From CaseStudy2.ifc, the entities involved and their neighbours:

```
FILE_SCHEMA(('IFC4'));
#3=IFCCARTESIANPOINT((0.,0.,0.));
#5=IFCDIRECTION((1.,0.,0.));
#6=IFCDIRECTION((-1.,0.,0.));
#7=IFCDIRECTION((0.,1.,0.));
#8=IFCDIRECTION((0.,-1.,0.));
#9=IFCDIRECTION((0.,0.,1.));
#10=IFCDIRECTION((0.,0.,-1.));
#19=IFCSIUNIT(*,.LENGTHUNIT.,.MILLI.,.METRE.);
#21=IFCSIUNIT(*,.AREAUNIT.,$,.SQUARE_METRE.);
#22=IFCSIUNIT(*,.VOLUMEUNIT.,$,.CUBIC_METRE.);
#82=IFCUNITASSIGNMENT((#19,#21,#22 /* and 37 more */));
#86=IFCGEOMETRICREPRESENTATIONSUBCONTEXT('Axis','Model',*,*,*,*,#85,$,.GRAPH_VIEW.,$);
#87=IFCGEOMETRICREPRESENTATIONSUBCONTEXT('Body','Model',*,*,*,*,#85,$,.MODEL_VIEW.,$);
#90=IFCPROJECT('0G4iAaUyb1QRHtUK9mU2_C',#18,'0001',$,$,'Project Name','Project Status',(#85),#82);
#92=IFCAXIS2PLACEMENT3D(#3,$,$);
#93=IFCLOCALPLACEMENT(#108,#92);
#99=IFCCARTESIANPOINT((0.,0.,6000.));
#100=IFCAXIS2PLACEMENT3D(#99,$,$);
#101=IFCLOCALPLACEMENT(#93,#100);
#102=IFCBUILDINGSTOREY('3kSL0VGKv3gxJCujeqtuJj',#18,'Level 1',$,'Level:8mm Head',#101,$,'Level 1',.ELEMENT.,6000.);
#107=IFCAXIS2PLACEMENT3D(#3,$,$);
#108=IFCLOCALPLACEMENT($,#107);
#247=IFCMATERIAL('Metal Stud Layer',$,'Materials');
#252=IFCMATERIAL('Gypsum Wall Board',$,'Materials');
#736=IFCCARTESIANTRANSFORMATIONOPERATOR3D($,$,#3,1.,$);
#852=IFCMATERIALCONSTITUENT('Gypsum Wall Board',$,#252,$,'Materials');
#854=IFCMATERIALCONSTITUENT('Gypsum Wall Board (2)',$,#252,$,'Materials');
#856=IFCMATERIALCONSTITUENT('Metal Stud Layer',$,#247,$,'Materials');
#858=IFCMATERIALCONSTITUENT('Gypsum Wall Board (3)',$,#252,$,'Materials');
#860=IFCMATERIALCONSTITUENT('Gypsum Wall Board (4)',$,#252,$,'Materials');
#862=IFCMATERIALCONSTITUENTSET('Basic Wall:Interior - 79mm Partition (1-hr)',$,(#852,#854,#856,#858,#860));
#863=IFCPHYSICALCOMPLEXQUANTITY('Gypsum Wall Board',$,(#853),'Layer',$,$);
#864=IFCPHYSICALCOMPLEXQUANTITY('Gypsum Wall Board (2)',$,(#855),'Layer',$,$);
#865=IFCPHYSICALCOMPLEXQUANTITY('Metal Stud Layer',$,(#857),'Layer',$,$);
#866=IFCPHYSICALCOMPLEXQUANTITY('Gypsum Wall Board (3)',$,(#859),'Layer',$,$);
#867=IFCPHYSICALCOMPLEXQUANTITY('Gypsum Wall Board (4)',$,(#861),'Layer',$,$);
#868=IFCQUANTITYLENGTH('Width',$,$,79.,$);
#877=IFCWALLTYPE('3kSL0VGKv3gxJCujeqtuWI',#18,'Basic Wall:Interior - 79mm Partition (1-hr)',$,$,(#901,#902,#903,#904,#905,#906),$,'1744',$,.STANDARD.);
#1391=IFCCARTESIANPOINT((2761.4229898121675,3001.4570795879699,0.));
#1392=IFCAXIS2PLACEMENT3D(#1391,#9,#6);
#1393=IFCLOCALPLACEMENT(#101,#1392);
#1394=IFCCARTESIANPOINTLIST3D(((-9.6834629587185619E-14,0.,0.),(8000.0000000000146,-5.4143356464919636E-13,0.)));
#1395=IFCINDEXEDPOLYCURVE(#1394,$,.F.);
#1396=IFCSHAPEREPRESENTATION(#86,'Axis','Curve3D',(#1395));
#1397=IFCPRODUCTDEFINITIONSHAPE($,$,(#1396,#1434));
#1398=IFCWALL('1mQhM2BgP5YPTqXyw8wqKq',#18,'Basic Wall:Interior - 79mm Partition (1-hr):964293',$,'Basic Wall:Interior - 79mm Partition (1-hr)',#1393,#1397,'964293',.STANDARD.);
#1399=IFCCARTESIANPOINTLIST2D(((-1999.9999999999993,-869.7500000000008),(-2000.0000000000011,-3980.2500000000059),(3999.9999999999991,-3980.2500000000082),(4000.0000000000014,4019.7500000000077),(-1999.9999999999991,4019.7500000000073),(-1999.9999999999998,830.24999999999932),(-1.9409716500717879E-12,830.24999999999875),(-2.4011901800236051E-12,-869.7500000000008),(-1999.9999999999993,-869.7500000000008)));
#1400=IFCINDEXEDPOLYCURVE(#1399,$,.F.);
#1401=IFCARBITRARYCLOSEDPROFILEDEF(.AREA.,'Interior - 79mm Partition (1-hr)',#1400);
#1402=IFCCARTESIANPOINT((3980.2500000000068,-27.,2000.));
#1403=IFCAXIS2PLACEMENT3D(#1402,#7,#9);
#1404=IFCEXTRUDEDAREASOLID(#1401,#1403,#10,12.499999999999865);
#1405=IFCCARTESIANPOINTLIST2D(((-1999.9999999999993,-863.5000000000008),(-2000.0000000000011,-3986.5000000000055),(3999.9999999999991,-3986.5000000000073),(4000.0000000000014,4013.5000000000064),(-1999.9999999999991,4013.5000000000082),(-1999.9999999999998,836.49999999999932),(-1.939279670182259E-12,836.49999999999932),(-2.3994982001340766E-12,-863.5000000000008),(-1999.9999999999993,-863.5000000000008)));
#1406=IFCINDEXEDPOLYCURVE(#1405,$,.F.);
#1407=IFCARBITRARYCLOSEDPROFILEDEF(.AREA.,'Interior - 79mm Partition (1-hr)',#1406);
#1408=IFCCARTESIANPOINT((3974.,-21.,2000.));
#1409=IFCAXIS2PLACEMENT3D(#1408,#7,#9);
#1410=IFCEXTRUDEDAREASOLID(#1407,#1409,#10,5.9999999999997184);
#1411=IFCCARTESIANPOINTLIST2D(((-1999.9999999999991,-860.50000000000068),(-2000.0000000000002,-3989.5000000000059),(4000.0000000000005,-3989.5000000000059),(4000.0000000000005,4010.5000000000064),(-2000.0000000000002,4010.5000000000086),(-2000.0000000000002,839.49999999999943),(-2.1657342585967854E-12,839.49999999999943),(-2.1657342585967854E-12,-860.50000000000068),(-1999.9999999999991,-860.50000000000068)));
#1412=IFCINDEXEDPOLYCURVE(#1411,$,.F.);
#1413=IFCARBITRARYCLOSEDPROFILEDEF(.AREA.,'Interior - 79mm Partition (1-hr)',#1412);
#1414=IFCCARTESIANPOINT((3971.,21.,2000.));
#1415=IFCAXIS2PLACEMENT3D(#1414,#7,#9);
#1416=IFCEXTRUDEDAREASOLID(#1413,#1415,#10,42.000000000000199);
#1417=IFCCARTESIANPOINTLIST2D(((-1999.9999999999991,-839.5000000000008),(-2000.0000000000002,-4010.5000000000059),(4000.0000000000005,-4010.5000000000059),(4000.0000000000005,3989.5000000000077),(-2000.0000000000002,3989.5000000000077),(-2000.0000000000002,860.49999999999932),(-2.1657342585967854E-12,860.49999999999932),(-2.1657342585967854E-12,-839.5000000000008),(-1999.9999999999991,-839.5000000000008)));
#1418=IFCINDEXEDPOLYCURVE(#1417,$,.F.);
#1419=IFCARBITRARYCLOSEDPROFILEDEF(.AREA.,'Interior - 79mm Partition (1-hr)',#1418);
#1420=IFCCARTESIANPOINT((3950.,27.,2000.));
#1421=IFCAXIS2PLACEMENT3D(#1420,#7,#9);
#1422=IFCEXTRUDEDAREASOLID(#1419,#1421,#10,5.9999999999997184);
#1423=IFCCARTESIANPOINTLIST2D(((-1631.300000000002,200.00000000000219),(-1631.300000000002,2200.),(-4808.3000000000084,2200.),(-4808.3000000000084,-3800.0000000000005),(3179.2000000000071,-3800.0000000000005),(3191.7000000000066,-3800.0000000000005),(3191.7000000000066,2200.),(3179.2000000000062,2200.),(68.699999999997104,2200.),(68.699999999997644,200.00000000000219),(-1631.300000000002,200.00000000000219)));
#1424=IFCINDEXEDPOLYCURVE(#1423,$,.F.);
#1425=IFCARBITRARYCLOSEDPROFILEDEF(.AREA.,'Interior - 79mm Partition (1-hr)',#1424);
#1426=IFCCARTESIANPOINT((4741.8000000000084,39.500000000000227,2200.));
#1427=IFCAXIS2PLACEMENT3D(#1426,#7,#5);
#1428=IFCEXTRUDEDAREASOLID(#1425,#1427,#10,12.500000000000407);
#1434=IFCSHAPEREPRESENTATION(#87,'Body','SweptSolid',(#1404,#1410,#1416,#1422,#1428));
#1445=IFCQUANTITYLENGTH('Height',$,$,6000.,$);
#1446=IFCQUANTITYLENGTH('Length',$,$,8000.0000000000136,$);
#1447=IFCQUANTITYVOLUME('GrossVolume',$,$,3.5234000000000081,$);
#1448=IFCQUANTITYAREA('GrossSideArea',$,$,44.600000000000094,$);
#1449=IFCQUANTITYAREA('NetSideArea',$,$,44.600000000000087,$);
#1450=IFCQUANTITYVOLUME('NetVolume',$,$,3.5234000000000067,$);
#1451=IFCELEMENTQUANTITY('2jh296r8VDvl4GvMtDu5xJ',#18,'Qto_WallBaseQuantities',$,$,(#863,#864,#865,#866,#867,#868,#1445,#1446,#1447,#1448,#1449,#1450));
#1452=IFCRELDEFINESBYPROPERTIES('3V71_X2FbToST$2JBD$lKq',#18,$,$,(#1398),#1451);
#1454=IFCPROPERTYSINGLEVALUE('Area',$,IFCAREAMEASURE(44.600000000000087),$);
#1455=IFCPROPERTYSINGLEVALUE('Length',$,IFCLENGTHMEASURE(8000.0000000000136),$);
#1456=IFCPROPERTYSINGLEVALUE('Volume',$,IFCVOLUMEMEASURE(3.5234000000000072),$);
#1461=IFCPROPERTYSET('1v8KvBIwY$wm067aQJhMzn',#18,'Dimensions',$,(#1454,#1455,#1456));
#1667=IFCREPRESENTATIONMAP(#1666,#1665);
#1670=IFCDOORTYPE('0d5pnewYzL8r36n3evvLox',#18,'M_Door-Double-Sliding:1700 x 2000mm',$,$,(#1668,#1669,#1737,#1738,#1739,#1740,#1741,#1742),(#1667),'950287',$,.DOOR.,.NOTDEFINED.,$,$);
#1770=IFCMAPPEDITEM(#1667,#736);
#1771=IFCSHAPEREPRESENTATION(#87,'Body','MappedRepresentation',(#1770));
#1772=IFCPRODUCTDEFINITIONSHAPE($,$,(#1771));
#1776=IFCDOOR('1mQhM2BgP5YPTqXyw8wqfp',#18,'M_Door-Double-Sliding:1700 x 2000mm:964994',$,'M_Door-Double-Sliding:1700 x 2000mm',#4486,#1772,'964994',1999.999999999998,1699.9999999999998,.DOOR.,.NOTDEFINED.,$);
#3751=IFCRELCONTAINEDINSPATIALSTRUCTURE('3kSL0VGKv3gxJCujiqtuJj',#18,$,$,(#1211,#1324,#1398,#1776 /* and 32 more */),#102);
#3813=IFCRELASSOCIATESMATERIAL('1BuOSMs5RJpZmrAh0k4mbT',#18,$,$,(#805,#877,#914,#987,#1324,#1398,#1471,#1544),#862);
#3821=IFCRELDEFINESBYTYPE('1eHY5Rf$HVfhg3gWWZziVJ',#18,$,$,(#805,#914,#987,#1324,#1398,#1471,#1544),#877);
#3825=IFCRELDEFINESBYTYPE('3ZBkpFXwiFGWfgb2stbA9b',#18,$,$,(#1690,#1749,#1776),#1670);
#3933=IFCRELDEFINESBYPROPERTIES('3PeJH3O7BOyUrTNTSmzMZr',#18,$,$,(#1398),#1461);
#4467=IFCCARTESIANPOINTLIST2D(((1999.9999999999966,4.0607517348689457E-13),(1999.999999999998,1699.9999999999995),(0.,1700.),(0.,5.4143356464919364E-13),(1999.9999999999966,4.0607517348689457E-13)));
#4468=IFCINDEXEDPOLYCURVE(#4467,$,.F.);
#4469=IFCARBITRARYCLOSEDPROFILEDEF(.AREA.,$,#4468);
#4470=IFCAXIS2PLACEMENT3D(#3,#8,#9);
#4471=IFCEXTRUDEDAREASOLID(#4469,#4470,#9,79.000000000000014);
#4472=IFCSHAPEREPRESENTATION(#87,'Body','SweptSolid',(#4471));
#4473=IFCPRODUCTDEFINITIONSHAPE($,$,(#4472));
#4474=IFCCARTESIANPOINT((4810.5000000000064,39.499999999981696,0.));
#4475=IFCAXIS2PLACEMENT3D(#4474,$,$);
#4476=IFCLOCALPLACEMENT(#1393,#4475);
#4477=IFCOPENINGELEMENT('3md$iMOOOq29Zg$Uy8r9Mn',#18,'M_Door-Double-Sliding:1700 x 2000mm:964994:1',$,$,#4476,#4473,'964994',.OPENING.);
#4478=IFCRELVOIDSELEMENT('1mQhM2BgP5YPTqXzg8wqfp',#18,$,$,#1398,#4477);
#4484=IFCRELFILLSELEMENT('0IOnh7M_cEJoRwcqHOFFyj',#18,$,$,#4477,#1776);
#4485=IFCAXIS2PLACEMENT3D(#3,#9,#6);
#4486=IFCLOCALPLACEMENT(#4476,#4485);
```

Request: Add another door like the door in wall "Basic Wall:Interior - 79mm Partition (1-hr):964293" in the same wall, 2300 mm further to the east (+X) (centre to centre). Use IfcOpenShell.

```python
import ifcopenshell
import ifcopenshell.api.feature
import ifcopenshell.api.geometry
import ifcopenshell.api.pset
import ifcopenshell.api.root
import ifcopenshell.geom
import ifcopenshell.util.element
import ifcopenshell.util.placement
import ifcopenshell.util.shape
import ifcopenshell.util.unit

model = ifcopenshell.open("CaseStudy2.ifc")
unit_scale = ifcopenshell.util.unit.calculate_unit_scale(model)
area_scale = ifcopenshell.util.unit.calculate_unit_scale(model, "AREAUNIT")
volume_scale = ifcopenshell.util.unit.calculate_unit_scale(model, "VOLUMEUNIT")
settings = ifcopenshell.geom.settings()


def volume(element):
    """Net volume in cubic metres, openings subtracted."""
    shape = ifcopenshell.geom.create_shape(settings, element)
    return ifcopenshell.util.shape.get_volume(shape.geometry)


def reuse_history(source, copy):
    """copy_class also copies each property set's owner history, people and application; keep the originals."""
    for rel in copy.IsDefinedBy:
        if rel.is_a("IfcRelDefinesByProperties") and (history := rel.RelatingPropertyDefinition.OwnerHistory):
            rel.RelatingPropertyDefinition.OwnerHistory = source.OwnerHistory
            ifcopenshell.util.element.remove_deep2(model, history)


door = model.by_id(1776)
opening = door.FillsVoids[0].RelatingOpeningElement
wall = opening.VoidsElements[0].RelatingBuildingElement
before = volume(wall)
shift = ifcopenshell.util.placement.get_local_placement(wall.ObjectPlacement)[:3, 0] * -2.3 / unit_scale

# copy_class copies the void relationship, type, container and properties, but no geometry.
new_opening = ifcopenshell.api.root.copy_class(model, product=opening)
new_opening.Representation = ifcopenshell.util.element.copy_deep(
    model, opening.Representation, exclude=["IfcGeometricRepresentationContext", "IfcRepresentationMap"]
)
new_opening.Name = "M_Door-Double-Sliding:1700 x 2000mm"
new_opening.Tag = None
reuse_history(opening, new_opening)
new_door = ifcopenshell.api.root.copy_class(model, product=door)
new_door.Representation = ifcopenshell.util.element.copy_deep(
    model, door.Representation, exclude=["IfcGeometricRepresentationContext", "IfcRepresentationMap"]
)
new_door.Name = "M_Door-Double-Sliding:1700 x 2000mm"
new_door.Tag = None
reuse_history(door, new_door)
ifcopenshell.api.feature.add_filling(model, opening=new_opening, element=new_door)

for old, new in ((opening, new_opening), (door, new_door)):
    matrix = ifcopenshell.util.placement.get_local_placement(old.ObjectPlacement)
    matrix[:3, 3] += shift
    ifcopenshell.api.geometry.edit_object_placement(model, product=new, matrix=matrix, is_si=False)

after = volume(wall)
thickness = 0.079  # wall thickness in metres

# Update the wall's stored quantities.
qto = model.by_id(ifcopenshell.util.element.get_pset(wall, "Qto_WallBaseQuantities", should_inherit=False)["id"])
ifcopenshell.api.pset.edit_qto(model, qto=qto, properties={
    "NetSideArea": after / thickness / area_scale,
    "NetVolume": after / volume_scale,
})
pset = model.by_id(ifcopenshell.util.element.get_pset(wall, "Dimensions", should_inherit=False)["id"])
ifcopenshell.api.pset.edit_pset(model, pset=pset, properties={
    "Area": model.create_entity("IfcAreaMeasure", after / thickness / area_scale),
    "Volume": model.create_entity("IfcVolumeMeasure", after / volume_scale),
})

print(f"wall volume {before:.3f} -> {after:.3f} m3")

model.write("CaseStudy2_updated.ifc")
```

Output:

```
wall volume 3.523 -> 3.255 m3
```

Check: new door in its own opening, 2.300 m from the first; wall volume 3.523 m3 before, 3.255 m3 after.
